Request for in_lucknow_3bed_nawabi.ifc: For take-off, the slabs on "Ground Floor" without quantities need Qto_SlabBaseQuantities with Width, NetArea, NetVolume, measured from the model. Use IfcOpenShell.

First a look at what the model holds.

```python
import ifcopenshell
import ifcopenshell.util.element
import ifcopenshell.util.unit

model = ifcopenshell.open("in_lucknow_3bed_nawabi.ifc")
print(model.schema)
for unit_type in ("LENGTHUNIT", "AREAUNIT", "VOLUMEUNIT"):
    print(unit_type, ifcopenshell.util.unit.calculate_unit_scale(model, unit_type))
storey = next(s for s in model.by_type("IfcBuildingStorey") if s.Name == "Ground Floor")
slabs = [e for e in ifcopenshell.util.element.get_decomposition(storey) if e.is_a("IfcSlab")]
for e in sorted(slabs, key=lambda e: e.id()):
    print(e.id(), e.is_a(), e.Name, list(ifcopenshell.util.element.get_psets(e, qtos_only=True)), sep=" | ")
```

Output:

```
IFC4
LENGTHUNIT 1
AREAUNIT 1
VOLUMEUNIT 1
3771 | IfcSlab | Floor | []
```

```python
import ifcopenshell
import ifcopenshell.api.pset
import ifcopenshell.geom
import ifcopenshell.util.element
import ifcopenshell.util.shape
import ifcopenshell.util.unit

model = ifcopenshell.open("in_lucknow_3bed_nawabi.ifc")
unit_scale = ifcopenshell.util.unit.calculate_unit_scale(model)
area_scale = ifcopenshell.util.unit.calculate_unit_scale(model, "AREAUNIT")
volume_scale = ifcopenshell.util.unit.calculate_unit_scale(model, "VOLUMEUNIT")
settings = ifcopenshell.geom.settings()

storey = next(s for s in model.by_type("IfcBuildingStorey") if s.Name == "Ground Floor")
slabs = [e for e in ifcopenshell.util.element.get_decomposition(storey) if e.is_a("IfcSlab")]

for e in sorted(slabs, key=lambda e: e.id()):
    if ifcopenshell.util.element.get_psets(e, qtos_only=True, should_inherit=False):
        continue
    # Geometry comes back in metres, in the element's own axes.
    shape = ifcopenshell.geom.create_shape(settings, e)
    values = {
        "Width": ifcopenshell.util.shape.get_z(shape.geometry) / unit_scale,
        "NetArea": ifcopenshell.util.shape.get_footprint_area(shape.geometry) / area_scale,
        "NetVolume": ifcopenshell.util.shape.get_volume(shape.geometry) / volume_scale,
    }
    qto = ifcopenshell.api.pset.add_qto(model, product=e, name="Qto_SlabBaseQuantities")
    ifcopenshell.api.pset.edit_qto(model, qto=qto, properties=values)
    print(e.id(), {k: round(v, 3) for k, v in values.items()})

model.write("in_lucknow_3bed_nawabi_updated.ifc")
```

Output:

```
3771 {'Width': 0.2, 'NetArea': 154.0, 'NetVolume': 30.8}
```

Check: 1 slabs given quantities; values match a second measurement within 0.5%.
